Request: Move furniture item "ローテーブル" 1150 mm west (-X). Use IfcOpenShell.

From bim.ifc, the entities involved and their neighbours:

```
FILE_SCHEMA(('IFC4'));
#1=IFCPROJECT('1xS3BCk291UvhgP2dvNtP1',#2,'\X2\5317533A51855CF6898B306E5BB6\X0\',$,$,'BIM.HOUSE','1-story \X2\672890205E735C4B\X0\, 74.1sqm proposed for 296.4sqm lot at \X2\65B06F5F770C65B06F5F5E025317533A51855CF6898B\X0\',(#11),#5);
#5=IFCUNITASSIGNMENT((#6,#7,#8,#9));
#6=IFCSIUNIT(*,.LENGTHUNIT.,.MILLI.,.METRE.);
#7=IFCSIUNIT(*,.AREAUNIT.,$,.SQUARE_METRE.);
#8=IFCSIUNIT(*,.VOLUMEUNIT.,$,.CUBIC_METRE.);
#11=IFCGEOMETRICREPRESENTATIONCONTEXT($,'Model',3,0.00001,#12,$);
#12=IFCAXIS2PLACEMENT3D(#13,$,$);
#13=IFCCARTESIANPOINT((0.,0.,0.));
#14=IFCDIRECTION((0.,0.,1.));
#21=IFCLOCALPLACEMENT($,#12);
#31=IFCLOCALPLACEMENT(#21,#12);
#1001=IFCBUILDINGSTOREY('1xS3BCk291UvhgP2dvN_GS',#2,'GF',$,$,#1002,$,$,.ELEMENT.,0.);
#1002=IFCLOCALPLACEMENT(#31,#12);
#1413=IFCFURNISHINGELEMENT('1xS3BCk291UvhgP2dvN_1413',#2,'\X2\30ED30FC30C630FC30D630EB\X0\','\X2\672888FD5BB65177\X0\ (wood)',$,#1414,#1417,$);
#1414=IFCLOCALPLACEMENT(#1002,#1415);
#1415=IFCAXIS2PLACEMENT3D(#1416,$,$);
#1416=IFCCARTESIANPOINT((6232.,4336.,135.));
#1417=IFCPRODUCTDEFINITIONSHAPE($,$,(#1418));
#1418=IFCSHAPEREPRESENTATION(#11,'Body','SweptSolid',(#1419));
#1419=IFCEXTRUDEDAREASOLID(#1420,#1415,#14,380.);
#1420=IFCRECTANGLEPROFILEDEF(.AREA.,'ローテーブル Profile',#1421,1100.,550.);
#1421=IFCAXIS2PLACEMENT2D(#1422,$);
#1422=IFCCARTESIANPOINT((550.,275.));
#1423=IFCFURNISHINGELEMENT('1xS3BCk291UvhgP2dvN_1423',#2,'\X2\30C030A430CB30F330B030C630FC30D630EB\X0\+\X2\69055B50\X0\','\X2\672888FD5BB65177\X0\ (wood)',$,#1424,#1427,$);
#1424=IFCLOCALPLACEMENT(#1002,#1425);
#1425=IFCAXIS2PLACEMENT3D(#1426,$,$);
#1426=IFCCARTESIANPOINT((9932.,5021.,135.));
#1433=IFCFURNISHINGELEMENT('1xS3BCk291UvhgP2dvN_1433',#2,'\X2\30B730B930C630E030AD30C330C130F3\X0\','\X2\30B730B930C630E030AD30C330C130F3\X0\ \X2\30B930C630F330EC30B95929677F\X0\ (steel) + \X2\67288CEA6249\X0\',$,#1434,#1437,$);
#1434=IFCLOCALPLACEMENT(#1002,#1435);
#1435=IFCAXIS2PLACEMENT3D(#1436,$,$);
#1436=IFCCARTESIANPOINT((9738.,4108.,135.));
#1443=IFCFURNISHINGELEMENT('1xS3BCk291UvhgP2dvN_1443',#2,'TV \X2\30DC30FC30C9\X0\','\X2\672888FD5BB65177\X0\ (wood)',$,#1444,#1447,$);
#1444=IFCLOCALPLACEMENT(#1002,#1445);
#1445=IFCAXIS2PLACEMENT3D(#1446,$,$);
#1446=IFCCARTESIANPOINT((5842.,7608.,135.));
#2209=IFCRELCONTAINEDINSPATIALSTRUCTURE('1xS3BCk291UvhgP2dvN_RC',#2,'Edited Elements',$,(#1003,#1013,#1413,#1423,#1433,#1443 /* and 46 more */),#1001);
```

```python
import ifcopenshell
import ifcopenshell.api.geometry
import ifcopenshell.util.placement
import ifcopenshell.util.unit

model = ifcopenshell.open("bim.ifc")
unit_scale = ifcopenshell.util.unit.calculate_unit_scale(model)

item = model.by_guid("1xS3BCk291UvhgP2dvN_1413")
matrix = ifcopenshell.util.placement.get_local_placement(item.ObjectPlacement)
matrix[0, 3] -= 1.15 / unit_scale
ifcopenshell.api.geometry.edit_object_placement(model, product=item, matrix=matrix, is_si=False)

print(ifcopenshell.util.placement.get_local_placement(item.ObjectPlacement).round(3) + 0.0)

model.write("bim_edited.ifc")
```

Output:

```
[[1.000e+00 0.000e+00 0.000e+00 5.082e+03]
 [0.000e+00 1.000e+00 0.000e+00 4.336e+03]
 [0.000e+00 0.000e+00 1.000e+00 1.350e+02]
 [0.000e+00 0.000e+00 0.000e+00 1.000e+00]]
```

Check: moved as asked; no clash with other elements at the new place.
